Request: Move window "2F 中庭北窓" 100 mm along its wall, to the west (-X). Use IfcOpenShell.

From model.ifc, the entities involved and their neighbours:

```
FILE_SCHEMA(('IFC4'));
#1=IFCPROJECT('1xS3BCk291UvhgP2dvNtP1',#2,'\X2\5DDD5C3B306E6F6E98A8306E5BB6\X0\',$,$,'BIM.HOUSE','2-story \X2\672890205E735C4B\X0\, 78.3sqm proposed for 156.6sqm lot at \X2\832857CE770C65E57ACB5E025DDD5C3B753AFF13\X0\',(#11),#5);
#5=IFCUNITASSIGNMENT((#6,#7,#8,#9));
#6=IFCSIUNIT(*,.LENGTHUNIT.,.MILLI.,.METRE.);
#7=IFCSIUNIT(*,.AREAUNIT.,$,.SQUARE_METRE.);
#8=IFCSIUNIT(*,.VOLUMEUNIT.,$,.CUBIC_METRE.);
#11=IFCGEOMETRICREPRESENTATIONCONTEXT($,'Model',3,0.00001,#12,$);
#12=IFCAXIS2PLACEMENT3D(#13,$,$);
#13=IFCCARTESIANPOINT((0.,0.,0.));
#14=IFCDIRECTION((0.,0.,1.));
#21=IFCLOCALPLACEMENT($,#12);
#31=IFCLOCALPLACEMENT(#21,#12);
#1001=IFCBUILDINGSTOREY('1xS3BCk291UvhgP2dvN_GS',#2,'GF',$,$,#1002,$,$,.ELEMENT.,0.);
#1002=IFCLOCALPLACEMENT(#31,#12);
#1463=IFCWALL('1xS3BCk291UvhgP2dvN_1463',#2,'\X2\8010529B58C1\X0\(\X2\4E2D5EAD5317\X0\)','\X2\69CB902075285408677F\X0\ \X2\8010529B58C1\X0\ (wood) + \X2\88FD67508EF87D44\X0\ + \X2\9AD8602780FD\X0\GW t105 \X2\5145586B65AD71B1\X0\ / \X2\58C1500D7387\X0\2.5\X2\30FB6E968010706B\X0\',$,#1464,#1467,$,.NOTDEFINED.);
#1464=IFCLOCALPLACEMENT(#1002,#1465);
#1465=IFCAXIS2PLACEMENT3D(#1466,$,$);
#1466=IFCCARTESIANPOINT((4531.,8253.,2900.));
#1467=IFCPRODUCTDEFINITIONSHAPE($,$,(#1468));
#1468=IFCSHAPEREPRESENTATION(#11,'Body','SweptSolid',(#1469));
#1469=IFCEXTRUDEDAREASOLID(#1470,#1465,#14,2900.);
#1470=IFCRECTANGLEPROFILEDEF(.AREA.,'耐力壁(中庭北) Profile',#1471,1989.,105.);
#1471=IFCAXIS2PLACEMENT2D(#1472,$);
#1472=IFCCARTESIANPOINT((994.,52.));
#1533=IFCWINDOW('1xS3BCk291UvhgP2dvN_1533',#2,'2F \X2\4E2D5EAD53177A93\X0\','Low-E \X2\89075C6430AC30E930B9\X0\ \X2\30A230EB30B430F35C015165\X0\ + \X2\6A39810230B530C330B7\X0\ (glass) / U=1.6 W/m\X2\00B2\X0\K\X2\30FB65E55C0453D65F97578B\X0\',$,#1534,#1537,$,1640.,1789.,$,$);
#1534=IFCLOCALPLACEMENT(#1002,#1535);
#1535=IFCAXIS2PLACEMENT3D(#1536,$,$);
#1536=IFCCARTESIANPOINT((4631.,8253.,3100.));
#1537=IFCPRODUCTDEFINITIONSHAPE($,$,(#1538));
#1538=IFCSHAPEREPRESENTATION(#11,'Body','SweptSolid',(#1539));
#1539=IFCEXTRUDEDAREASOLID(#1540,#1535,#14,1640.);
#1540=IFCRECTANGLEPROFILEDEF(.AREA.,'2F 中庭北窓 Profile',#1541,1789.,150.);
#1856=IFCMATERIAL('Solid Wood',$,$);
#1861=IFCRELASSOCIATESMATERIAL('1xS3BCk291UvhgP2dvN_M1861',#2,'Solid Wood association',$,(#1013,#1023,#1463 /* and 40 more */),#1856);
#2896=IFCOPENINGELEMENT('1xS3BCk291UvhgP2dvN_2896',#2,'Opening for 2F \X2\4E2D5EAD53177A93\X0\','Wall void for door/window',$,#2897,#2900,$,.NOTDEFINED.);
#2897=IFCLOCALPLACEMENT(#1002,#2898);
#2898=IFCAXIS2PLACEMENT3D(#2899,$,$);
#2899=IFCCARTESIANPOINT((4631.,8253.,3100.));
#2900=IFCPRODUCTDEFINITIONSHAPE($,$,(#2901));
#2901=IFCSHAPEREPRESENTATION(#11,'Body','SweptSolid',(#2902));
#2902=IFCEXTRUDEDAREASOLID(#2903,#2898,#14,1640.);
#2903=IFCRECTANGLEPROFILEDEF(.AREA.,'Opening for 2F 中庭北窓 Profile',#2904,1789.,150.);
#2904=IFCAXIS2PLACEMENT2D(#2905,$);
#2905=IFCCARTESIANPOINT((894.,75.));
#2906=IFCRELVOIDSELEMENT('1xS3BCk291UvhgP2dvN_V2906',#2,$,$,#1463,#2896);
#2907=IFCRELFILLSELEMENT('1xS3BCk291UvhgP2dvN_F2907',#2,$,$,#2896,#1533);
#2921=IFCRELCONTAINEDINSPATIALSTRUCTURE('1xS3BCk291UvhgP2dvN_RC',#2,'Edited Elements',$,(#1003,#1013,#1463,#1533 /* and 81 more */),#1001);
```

```python
import ifcopenshell
import ifcopenshell.api.geometry
import ifcopenshell.util.placement
import ifcopenshell.util.unit

model = ifcopenshell.open("model.ifc")
unit_scale = ifcopenshell.util.unit.calculate_unit_scale(model)

window = model.by_guid("1xS3BCk291UvhgP2dvN_1533")
opening = window.FillsVoids[0].RelatingOpeningElement
wall = opening.VoidsElements[0].RelatingBuildingElement

wall_matrix = ifcopenshell.util.placement.get_local_placement(wall.ObjectPlacement)
shift = wall_matrix[:3, 0] * -0.1 / unit_scale
before = ifcopenshell.util.placement.get_local_placement(window.ObjectPlacement)[:3, 3].copy()

# The window is not placed relative to its opening, so move both.
for product in (opening, window):
    matrix = ifcopenshell.util.placement.get_local_placement(product.ObjectPlacement)
    matrix[:3, 3] += shift
    ifcopenshell.api.geometry.edit_object_placement(model, product=product, matrix=matrix, is_si=False)

after = ifcopenshell.util.placement.get_local_placement(window.ObjectPlacement)[:3, 3]
print("window moved by", (after - before).round(3) + 0.0)

model.write("model_v2.ifc")
```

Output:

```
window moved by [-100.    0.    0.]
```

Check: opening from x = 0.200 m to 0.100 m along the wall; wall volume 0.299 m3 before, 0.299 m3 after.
